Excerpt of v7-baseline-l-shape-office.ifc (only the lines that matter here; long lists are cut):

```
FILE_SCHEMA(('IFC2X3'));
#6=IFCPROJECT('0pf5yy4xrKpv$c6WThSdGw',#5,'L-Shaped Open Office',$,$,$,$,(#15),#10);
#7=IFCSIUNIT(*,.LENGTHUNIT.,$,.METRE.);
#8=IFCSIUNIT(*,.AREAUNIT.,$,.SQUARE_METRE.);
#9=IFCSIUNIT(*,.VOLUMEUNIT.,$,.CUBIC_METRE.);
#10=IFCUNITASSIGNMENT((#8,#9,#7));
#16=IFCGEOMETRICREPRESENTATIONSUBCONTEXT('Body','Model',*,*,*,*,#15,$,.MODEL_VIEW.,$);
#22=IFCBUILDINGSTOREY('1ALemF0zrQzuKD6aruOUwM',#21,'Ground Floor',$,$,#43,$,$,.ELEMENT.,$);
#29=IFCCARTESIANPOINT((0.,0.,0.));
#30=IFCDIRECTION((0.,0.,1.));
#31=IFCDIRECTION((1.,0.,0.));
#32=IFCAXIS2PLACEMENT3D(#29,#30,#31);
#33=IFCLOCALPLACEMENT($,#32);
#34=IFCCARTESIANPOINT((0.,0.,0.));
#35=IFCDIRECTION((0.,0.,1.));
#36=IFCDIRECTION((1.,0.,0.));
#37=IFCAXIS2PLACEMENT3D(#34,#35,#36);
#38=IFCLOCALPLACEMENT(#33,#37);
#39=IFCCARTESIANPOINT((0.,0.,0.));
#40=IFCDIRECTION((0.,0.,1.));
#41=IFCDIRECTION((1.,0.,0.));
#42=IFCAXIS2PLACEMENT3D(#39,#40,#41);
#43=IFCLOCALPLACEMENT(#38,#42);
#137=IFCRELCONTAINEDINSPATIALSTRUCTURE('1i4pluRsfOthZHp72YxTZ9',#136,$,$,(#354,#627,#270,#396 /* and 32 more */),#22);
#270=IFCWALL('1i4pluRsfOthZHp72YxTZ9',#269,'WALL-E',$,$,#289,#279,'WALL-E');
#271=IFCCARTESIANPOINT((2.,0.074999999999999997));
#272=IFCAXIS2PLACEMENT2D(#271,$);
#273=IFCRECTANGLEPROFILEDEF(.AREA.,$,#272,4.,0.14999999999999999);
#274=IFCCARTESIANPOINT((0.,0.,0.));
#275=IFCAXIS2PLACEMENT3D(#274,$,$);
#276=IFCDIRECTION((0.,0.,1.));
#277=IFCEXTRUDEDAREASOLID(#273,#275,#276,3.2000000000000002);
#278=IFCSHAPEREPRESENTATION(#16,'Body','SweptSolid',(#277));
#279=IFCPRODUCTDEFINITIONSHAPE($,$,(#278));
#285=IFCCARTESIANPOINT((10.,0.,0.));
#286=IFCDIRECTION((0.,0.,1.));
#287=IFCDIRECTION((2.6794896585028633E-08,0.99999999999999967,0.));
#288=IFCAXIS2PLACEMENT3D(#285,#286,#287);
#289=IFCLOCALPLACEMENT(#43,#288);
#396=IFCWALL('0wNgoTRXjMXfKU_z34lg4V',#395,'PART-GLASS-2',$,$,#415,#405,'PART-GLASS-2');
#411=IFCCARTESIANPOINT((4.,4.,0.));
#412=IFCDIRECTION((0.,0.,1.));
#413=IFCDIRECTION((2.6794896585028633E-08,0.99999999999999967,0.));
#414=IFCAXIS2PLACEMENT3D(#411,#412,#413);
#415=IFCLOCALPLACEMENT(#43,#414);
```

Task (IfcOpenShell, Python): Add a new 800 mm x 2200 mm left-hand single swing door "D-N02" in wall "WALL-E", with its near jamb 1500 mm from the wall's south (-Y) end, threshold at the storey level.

```python
import numpy as np
import ifcopenshell
import ifcopenshell.api.feature
import ifcopenshell.api.geometry
import ifcopenshell.api.root
import ifcopenshell.api.spatial
import ifcopenshell.api.type
import ifcopenshell.geom
import ifcopenshell.util.element
import ifcopenshell.util.placement
import ifcopenshell.util.representation
import ifcopenshell.util.shape
import ifcopenshell.util.unit

model = ifcopenshell.open("v7-baseline-l-shape-office.ifc")
unit_scale = ifcopenshell.util.unit.calculate_unit_scale(model)
settings = ifcopenshell.geom.settings()


def volume(element):
    """Net volume in cubic metres, openings subtracted."""
    shape = ifcopenshell.geom.create_shape(settings, element)
    return ifcopenshell.util.shape.get_volume(shape.geometry)


wall = model.by_id(270)
storey = ifcopenshell.util.element.get_container(wall, ifc_class="IfcBuildingStorey")
context = ifcopenshell.util.representation.get_context(model, "Model", "Body", "MODEL_VIEW")
before = volume(wall)

width, height, from_end, sill = 0.8, 2.2, 1.5, 0.0  # metres

# The wall runs along its own X axis, and the end named is its -X end.
wall_shape = ifcopenshell.geom.create_shape(settings, wall)
x, y, z = ifcopenshell.util.shape.get_vertices(wall_shape.geometry).T
start = x.min() + from_end
face, thickness = float(y.min()), float(y.max() - y.min())
wall_matrix = ifcopenshell.util.placement.get_local_placement(wall.ObjectPlacement)
level = ifcopenshell.util.placement.get_local_placement(storey.ObjectPlacement)[2, 3]


def in_wall(x, y):
    """Placement at x, y metres in the wall's axes, at sill height."""
    matrix = wall_matrix.copy()
    matrix[:, 3] = wall_matrix @ np.array([x / unit_scale, y / unit_scale, 0.0, 1.0])
    matrix[2, 3] = level + sill / unit_scale
    return matrix


# Opening: a box that overshoots both wall faces by 50 mm.
opening = ifcopenshell.api.root.create_entity(model, ifc_class="IfcOpeningElement")
box = ifcopenshell.api.geometry.add_wall_representation(
    model, context=context, length=width, height=height, thickness=thickness + 0.1
)
ifcopenshell.api.geometry.assign_representation(model, product=opening, representation=box)
ifcopenshell.api.geometry.edit_object_placement(model, product=opening, matrix=in_wall(start, face - 0.05), is_si=False)
ifcopenshell.api.feature.add_feature(model, feature=opening, element=wall)

door = ifcopenshell.api.root.create_entity(model, ifc_class="IfcDoor", name="D-N02")
door.OverallWidth, door.OverallHeight = width / unit_scale, height / unit_scale
body = ifcopenshell.api.geometry.add_door_representation(
    model,
    context=context,
    overall_width=door.OverallWidth,
    overall_height=door.OverallHeight,
    operation_type="SINGLE_SWING_LEFT",
    lining_properties={"LiningDepth": thickness / unit_scale, "ThresholdDepth": thickness / unit_scale},
)
ifcopenshell.api.geometry.assign_representation(model, product=door, representation=body)
ifcopenshell.api.spatial.assign_container(model, products=[door], relating_structure=storey)
fills = ifcopenshell.api.feature.add_filling(model, opening=opening, element=door)
fills.OwnerHistory = door.OwnerHistory  # required in IFC2X3

# IFC2X3 keeps the operation on the door style.
style = ifcopenshell.api.root.create_entity(model, ifc_class="IfcDoorStyle", name="D-N02")
style.OperationType, style.ConstructionType = "SINGLE_SWING_LEFT", "NOTDEFINED"
style.ParameterTakesPrecedence = style.Sizeable = False
ifcopenshell.api.type.assign_type(model, related_objects=[door], relating_type=style)

# The lining spans the wall, so the door starts at the wall face.
ifcopenshell.api.geometry.edit_object_placement(model, product=door, matrix=in_wall(start, face), is_si=False)

after = volume(wall)

print(f"wall volume {before:.3f} -> {after:.3f} m3")

model.write("v7-baseline-l-shape-office_updated.ifc")
```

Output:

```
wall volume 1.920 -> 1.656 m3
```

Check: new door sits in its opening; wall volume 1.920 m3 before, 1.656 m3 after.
